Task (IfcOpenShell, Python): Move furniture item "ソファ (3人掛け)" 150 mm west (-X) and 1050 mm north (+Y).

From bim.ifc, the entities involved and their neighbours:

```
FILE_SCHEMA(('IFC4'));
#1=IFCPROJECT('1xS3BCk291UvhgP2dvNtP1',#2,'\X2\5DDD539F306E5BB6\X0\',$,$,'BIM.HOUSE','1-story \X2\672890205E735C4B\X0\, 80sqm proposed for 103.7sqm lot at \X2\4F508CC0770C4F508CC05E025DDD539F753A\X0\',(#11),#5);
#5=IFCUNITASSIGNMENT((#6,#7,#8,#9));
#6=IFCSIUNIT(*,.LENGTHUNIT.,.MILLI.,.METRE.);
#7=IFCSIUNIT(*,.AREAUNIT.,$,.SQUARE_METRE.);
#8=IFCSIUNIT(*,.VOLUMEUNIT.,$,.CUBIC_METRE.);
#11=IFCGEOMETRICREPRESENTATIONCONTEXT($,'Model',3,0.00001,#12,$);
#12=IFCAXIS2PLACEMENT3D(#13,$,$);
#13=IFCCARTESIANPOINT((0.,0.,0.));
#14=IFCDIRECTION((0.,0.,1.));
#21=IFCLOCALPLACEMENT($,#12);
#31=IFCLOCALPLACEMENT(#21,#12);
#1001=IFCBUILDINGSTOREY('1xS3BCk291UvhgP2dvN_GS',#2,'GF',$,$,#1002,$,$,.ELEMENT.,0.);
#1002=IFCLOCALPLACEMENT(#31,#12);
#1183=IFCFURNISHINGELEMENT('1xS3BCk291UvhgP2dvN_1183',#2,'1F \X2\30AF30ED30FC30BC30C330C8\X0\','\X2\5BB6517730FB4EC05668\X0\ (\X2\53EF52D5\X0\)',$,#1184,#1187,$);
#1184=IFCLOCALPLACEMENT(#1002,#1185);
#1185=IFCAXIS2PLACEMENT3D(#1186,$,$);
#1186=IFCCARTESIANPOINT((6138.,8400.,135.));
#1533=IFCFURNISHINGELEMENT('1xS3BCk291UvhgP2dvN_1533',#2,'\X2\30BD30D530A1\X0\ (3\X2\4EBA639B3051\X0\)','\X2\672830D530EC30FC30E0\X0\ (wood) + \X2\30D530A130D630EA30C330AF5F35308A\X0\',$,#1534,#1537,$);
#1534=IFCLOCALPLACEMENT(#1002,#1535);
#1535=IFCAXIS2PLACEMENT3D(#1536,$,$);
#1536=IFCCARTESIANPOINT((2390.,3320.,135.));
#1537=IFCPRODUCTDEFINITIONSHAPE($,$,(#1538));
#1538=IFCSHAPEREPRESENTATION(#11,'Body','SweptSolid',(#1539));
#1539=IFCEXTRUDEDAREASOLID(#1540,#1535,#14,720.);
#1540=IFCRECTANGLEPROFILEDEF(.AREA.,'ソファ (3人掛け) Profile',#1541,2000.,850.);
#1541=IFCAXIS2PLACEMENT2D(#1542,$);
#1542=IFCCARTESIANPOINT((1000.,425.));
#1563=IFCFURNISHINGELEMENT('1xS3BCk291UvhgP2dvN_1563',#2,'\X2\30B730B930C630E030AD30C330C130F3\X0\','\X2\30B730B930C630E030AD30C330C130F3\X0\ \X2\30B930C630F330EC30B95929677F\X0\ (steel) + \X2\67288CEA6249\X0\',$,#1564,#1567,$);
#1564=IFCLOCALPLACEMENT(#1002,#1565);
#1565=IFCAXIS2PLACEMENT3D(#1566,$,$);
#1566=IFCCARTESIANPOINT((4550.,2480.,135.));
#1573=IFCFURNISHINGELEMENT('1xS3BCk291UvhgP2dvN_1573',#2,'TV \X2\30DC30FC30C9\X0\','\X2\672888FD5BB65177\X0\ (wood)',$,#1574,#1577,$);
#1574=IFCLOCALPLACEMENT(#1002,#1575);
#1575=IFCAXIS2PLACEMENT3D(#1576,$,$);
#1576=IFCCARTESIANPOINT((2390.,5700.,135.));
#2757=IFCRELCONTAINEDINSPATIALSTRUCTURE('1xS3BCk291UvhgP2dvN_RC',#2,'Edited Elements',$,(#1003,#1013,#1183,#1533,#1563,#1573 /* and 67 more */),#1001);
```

```python
import ifcopenshell
import ifcopenshell.api.geometry
import ifcopenshell.util.placement
import ifcopenshell.util.unit

model = ifcopenshell.open("bim.ifc")
unit_scale = ifcopenshell.util.unit.calculate_unit_scale(model)

item = model.by_id(1533)
matrix = ifcopenshell.util.placement.get_local_placement(item.ObjectPlacement)
matrix[0, 3] -= 0.15 / unit_scale
matrix[1, 3] += 1.05 / unit_scale
ifcopenshell.api.geometry.edit_object_placement(model, product=item, matrix=matrix, is_si=False)

print(ifcopenshell.util.placement.get_local_placement(item.ObjectPlacement).round(3) + 0.0)

model.write("bim_v2.ifc")
```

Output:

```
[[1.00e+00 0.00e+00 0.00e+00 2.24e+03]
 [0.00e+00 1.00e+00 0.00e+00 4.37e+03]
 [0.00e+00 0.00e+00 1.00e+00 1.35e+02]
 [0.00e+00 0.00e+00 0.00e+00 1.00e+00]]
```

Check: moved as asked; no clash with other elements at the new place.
